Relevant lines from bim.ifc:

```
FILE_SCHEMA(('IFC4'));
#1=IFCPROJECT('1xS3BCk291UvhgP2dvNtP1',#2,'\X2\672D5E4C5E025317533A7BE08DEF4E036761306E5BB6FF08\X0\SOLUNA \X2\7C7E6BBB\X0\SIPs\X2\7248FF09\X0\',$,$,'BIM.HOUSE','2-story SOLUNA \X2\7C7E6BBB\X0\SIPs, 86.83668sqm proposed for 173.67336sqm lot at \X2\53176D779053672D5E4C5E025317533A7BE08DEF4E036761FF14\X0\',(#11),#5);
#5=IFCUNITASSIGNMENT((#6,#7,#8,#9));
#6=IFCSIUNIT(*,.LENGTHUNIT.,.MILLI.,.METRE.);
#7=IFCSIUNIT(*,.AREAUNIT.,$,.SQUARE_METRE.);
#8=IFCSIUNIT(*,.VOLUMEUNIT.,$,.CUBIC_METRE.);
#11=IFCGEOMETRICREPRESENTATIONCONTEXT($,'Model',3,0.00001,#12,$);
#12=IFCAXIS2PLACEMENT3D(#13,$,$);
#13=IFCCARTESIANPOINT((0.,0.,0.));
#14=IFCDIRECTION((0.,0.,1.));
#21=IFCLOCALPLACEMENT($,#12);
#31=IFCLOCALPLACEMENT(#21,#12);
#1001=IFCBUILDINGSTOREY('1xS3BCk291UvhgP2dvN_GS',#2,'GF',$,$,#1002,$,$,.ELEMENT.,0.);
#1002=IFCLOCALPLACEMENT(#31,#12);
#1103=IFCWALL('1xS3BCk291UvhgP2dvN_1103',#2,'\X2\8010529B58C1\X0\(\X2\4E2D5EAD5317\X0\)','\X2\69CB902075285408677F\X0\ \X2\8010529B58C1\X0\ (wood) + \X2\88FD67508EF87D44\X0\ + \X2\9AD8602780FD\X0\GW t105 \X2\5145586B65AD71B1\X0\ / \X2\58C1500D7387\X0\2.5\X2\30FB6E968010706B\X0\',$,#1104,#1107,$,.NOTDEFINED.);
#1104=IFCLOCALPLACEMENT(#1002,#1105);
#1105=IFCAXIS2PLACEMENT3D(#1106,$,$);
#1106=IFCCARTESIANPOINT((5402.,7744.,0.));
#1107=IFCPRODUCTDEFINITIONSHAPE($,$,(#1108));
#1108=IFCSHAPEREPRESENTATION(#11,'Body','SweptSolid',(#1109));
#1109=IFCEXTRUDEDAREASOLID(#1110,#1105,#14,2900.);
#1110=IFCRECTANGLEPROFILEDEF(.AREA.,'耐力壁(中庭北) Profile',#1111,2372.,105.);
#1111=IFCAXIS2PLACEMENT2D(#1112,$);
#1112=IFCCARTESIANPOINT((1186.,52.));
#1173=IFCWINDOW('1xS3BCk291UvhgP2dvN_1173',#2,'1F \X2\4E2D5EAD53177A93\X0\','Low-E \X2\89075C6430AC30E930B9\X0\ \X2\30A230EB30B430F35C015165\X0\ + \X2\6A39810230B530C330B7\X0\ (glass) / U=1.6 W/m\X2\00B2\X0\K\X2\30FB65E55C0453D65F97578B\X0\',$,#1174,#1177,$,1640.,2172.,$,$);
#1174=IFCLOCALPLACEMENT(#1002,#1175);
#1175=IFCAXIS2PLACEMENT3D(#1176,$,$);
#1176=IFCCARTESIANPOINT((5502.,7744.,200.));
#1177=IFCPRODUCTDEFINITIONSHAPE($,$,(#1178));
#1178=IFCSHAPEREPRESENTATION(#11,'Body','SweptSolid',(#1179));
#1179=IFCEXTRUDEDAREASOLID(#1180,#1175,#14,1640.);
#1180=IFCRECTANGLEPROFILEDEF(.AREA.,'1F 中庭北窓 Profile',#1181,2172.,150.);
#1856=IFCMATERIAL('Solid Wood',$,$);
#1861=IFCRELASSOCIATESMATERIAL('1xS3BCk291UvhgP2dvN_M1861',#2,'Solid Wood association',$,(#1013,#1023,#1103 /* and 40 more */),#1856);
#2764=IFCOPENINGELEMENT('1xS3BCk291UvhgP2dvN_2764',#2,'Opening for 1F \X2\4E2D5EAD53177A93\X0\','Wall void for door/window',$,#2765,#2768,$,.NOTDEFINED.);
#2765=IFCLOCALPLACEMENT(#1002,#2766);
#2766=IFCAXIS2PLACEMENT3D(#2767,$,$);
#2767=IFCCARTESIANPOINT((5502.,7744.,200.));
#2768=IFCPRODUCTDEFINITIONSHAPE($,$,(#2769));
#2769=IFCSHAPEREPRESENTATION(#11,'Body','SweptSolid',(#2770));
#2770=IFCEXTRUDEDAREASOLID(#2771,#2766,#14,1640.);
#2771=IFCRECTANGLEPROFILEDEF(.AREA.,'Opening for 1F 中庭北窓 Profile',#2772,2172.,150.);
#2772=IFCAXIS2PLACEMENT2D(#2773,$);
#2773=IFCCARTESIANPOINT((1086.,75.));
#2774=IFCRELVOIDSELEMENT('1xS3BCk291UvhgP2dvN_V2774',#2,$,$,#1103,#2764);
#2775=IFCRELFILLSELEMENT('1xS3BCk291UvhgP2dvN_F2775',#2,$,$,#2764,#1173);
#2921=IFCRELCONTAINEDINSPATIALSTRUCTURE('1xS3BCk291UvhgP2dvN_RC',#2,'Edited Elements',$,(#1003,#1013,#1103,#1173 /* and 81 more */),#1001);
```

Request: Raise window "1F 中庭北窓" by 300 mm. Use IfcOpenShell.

```python
import numpy as np
import ifcopenshell
import ifcopenshell.api.geometry
import ifcopenshell.util.placement
import ifcopenshell.util.unit

model = ifcopenshell.open("bim.ifc")
unit_scale = ifcopenshell.util.unit.calculate_unit_scale(model)

window = model.by_guid("1xS3BCk291UvhgP2dvN_1173")
opening = window.FillsVoids[0].RelatingOpeningElement
dz = 0.3 / unit_scale

shift = np.array([0.0, 0.0, dz])
# The window is not placed relative to its opening, so move both.
for product in (opening, window):
    matrix = ifcopenshell.util.placement.get_local_placement(product.ObjectPlacement)
    matrix[:3, 3] += shift
    ifcopenshell.api.geometry.edit_object_placement(model, product=product, matrix=matrix, is_si=False)

print(f"moved by {dz * unit_scale:+.3f} m")

model.write("bim_edited.ifc")
```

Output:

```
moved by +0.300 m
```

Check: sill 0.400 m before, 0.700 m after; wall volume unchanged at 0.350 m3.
